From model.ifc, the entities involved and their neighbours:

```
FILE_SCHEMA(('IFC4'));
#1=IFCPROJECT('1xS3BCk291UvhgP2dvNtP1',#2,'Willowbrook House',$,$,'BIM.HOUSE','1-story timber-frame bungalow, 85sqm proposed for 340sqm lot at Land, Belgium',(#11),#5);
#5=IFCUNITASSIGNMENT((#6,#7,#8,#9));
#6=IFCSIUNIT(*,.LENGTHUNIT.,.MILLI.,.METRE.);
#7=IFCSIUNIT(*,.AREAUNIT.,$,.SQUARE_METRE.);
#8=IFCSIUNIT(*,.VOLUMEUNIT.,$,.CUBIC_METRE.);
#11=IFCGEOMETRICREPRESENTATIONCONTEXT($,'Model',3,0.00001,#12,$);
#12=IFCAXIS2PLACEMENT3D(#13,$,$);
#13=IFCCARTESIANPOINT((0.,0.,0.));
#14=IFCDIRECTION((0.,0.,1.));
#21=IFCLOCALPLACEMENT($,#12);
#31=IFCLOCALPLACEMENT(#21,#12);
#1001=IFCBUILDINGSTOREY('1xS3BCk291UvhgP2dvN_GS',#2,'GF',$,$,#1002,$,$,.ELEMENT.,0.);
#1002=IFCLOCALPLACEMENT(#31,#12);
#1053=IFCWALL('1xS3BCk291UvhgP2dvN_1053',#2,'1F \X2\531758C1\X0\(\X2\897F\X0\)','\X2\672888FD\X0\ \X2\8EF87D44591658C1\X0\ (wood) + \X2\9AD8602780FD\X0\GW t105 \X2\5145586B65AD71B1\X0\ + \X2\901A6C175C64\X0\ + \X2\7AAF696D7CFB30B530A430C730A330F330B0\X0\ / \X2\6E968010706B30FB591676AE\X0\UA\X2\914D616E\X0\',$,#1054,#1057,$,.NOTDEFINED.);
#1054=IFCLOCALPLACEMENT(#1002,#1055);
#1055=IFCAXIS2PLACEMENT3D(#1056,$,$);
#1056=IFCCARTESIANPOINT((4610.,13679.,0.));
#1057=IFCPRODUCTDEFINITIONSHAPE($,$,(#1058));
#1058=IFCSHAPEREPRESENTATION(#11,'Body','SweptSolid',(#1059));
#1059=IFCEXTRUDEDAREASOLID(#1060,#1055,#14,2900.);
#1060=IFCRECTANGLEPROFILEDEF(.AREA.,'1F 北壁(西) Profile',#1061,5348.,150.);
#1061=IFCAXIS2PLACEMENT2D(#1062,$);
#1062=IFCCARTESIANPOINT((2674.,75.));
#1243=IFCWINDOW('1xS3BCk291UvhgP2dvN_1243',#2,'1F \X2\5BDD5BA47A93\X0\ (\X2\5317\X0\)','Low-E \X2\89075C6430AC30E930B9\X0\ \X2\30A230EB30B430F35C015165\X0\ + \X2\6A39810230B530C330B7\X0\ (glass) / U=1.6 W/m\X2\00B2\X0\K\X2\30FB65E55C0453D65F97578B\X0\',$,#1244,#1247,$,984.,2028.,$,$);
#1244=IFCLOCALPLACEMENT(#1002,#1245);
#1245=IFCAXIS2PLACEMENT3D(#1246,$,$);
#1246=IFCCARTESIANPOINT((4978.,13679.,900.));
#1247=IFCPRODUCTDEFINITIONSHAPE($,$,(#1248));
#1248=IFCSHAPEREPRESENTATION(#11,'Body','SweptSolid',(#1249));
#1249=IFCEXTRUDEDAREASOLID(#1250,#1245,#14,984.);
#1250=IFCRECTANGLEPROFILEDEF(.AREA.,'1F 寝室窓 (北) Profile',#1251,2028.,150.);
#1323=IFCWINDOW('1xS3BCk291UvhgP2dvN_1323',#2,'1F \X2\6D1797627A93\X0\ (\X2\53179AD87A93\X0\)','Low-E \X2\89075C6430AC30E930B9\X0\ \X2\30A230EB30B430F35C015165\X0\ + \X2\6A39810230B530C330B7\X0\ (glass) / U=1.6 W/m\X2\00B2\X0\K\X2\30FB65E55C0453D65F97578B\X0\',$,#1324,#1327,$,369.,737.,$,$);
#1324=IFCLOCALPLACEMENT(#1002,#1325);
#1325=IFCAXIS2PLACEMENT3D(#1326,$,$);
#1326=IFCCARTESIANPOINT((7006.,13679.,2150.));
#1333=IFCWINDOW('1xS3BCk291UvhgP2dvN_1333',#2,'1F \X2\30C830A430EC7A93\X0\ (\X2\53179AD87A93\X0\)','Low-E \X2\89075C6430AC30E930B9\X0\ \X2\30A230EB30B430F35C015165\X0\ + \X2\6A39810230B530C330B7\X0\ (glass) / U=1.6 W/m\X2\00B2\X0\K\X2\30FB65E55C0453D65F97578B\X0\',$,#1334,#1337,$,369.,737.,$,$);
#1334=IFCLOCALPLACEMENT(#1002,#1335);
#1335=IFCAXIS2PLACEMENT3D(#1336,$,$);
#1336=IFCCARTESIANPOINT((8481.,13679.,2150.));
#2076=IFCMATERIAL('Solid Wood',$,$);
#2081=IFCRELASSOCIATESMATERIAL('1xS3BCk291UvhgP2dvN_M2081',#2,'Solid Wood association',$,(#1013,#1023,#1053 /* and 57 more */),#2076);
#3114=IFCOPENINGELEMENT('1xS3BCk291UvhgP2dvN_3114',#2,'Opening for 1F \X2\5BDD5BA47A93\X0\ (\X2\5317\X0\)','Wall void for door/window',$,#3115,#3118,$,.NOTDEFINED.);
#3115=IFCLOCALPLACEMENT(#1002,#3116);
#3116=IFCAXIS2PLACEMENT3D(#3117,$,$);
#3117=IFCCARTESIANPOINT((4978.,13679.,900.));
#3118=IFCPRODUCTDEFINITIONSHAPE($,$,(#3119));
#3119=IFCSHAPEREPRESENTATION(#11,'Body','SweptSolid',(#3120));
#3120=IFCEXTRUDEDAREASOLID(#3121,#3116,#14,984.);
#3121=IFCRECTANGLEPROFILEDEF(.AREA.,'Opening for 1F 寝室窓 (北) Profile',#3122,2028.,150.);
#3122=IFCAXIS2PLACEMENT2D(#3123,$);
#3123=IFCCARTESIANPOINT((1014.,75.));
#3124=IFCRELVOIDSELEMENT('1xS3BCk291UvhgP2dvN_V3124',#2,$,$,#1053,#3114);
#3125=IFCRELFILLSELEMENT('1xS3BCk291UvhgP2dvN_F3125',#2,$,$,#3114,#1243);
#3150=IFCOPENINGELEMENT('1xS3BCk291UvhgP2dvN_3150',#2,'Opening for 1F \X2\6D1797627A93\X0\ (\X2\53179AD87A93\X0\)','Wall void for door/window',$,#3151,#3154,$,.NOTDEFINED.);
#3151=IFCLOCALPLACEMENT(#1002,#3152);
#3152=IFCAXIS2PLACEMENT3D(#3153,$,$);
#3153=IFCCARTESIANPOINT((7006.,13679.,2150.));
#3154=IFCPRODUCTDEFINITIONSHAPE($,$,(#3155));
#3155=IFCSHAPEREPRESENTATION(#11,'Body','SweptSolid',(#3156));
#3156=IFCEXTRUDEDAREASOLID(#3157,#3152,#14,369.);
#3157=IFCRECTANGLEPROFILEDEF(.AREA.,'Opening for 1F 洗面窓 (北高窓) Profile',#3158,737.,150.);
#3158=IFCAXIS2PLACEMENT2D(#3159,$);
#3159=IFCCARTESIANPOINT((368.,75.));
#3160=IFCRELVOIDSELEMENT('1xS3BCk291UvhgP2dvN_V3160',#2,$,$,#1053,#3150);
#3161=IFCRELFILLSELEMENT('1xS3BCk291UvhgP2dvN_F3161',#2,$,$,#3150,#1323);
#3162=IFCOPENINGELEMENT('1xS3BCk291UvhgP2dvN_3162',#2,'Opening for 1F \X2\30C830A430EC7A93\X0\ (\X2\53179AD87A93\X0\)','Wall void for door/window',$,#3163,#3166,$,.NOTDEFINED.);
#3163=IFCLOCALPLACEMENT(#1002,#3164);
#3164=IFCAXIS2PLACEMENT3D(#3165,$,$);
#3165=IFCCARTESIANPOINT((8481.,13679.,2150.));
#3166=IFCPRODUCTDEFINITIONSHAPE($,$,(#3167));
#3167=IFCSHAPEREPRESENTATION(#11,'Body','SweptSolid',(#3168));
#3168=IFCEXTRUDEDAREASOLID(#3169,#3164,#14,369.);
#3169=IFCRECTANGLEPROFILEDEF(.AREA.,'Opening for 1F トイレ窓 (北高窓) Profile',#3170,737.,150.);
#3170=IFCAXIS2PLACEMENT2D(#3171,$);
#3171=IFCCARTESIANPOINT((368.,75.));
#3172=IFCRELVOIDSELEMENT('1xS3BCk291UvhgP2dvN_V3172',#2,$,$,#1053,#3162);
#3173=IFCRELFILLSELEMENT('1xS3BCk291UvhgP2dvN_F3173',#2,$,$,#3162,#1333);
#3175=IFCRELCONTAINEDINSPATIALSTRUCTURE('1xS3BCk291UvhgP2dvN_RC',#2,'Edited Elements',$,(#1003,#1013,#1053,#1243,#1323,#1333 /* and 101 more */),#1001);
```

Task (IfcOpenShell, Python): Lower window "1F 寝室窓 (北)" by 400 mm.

```python
import numpy as np
import ifcopenshell
import ifcopenshell.api.geometry
import ifcopenshell.util.placement
import ifcopenshell.util.unit

model = ifcopenshell.open("model.ifc")
unit_scale = ifcopenshell.util.unit.calculate_unit_scale(model)

window = model.by_id(1243)
opening = window.FillsVoids[0].RelatingOpeningElement
dz = -0.4 / unit_scale

shift = np.array([0.0, 0.0, dz])
# The window is not placed relative to its opening, so move both.
for product in (opening, window):
    matrix = ifcopenshell.util.placement.get_local_placement(product.ObjectPlacement)
    matrix[:3, 3] += shift
    ifcopenshell.api.geometry.edit_object_placement(model, product=product, matrix=matrix, is_si=False)

print(f"moved by {dz * unit_scale:+.3f} m")

model.write("model_rev.ifc")
```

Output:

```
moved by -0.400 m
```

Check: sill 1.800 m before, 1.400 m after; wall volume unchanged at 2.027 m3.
